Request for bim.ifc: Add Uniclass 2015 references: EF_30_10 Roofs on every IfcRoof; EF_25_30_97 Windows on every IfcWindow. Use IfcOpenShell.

First a look at what the model holds.

```python
import ifcopenshell

model = ifcopenshell.open("bim.ifc")
print(model.schema)
print("classifications:", [c.Name for c in model.by_type("IfcClassification")])
for ifc_class in ("IfcDoor", "IfcRoof", "IfcStair", "IfcWall", "IfcWindow"):
    print(ifc_class, len(model.by_type(ifc_class)))
```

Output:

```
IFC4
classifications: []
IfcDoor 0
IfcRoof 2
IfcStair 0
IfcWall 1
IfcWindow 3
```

```python
import ifcopenshell
import ifcopenshell.api.classification

model = ifcopenshell.open("bim.ifc")

system = ifcopenshell.api.classification.add_classification(model, classification="Uniclass 2015")

codes = {
    "IfcRoof": ("EF_30_10", "Roofs"),
    "IfcWindow": ("EF_25_30_97", "Windows"),
}
for ifc_class, (code, name) in codes.items():
    products = model.by_type(ifc_class)
    ifcopenshell.api.classification.add_reference(
        model, products=products, classification=system, identification=code, name=name
    )
    print(code, len(products))

model.write("bim_updated.ifc")
```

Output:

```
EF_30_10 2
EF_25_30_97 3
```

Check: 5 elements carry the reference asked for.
